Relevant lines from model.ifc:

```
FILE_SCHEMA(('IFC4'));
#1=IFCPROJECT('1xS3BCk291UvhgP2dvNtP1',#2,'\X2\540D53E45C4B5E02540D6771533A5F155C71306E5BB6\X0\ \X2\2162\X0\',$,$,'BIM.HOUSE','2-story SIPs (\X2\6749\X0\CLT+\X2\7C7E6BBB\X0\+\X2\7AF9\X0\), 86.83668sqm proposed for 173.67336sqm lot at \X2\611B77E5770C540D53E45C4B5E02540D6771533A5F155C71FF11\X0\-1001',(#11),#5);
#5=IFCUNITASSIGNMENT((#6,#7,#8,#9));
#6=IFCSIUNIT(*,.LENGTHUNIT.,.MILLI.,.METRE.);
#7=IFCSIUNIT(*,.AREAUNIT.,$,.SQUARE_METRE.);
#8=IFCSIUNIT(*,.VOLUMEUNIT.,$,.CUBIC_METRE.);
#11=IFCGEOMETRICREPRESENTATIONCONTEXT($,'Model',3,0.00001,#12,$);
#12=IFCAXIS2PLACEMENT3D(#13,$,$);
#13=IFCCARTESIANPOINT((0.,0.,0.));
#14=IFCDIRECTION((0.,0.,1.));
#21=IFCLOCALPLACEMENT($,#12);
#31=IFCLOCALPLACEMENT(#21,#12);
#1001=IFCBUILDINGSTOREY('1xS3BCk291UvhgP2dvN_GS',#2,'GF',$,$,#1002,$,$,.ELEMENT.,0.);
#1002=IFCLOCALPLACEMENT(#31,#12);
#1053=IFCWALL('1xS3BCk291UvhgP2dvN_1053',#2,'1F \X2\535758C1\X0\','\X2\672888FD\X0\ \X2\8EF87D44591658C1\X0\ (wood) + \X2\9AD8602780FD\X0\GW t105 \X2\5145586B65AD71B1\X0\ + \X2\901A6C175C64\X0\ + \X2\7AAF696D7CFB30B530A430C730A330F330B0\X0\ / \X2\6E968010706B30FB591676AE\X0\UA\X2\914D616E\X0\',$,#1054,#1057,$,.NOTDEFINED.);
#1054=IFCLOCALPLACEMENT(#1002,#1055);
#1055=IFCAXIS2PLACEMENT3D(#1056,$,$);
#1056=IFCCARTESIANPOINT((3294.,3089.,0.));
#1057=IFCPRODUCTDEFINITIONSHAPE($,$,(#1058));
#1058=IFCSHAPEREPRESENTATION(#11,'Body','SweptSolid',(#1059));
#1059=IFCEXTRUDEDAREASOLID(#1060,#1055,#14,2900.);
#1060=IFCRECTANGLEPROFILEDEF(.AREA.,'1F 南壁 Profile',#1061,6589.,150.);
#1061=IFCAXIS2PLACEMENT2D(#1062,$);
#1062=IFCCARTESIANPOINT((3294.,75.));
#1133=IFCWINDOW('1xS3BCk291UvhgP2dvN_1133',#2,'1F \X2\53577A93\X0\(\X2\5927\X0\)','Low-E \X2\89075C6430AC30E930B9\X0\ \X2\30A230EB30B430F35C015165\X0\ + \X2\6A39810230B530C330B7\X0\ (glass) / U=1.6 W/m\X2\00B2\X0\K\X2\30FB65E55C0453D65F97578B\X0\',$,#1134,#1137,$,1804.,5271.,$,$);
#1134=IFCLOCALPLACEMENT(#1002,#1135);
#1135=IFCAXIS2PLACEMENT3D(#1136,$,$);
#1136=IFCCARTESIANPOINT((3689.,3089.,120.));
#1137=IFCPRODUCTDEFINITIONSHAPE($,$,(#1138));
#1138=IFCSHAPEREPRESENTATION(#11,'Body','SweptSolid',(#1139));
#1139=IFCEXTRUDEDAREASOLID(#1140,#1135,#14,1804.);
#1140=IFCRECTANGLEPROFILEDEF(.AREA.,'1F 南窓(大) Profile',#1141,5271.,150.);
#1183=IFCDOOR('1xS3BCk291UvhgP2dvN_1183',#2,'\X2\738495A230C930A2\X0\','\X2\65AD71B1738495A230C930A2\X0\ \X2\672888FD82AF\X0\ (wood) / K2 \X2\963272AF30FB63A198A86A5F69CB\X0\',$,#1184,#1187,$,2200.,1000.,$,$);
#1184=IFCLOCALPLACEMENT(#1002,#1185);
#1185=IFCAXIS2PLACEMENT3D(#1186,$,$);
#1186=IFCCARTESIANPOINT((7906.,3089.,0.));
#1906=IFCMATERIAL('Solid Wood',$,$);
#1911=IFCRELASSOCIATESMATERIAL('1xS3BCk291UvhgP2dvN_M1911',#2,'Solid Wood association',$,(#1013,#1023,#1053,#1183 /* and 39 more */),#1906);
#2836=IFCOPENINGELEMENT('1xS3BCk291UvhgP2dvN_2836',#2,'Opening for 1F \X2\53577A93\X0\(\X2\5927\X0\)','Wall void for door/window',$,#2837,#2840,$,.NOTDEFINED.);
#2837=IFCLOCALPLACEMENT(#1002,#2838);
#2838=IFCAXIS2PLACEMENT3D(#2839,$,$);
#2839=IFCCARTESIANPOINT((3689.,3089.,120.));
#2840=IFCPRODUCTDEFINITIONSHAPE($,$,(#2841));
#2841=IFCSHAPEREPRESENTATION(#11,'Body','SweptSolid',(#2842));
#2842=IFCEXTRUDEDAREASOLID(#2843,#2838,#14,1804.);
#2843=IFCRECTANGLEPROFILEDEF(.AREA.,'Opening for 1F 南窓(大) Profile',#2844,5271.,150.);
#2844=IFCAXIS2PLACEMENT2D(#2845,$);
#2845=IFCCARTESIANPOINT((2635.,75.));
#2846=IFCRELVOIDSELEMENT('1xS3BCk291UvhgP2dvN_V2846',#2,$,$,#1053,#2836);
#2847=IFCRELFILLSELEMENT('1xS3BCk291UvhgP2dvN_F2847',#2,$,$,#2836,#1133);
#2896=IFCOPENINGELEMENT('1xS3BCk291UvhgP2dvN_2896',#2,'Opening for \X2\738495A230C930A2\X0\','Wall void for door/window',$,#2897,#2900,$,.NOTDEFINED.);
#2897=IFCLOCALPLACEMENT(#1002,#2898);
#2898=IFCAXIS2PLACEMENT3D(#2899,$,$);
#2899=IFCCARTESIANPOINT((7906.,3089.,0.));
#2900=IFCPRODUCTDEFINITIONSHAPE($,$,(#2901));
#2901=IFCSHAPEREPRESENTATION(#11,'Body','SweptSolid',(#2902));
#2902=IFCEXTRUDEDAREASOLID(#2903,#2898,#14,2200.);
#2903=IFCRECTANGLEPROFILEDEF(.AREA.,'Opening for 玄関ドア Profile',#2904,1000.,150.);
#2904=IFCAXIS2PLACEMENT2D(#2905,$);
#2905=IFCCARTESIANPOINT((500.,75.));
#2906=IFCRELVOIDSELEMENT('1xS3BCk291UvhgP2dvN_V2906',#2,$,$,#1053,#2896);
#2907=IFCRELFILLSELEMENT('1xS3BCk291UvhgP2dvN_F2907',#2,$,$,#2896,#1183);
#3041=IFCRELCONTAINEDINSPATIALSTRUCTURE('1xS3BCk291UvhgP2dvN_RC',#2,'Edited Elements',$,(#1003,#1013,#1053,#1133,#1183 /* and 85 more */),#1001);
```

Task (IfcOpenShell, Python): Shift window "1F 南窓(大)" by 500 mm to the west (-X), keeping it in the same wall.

```python
import ifcopenshell
import ifcopenshell.api.geometry
import ifcopenshell.util.placement
import ifcopenshell.util.unit

model = ifcopenshell.open("model.ifc")
unit_scale = ifcopenshell.util.unit.calculate_unit_scale(model)

window = model.by_guid("1xS3BCk291UvhgP2dvN_1133")
opening = window.FillsVoids[0].RelatingOpeningElement
wall = opening.VoidsElements[0].RelatingBuildingElement

wall_matrix = ifcopenshell.util.placement.get_local_placement(wall.ObjectPlacement)
shift = wall_matrix[:3, 0] * -0.5 / unit_scale
before = ifcopenshell.util.placement.get_local_placement(window.ObjectPlacement)[:3, 3].copy()

# The window is not placed relative to its opening, so move both.
for product in (opening, window):
    matrix = ifcopenshell.util.placement.get_local_placement(product.ObjectPlacement)
    matrix[:3, 3] += shift
    ifcopenshell.api.geometry.edit_object_placement(model, product=product, matrix=matrix, is_si=False)

after = ifcopenshell.util.placement.get_local_placement(window.ObjectPlacement)[:3, 3]
print("window moved by", (after - before).round(3) + 0.0)

model.write("model_v2.ifc")
```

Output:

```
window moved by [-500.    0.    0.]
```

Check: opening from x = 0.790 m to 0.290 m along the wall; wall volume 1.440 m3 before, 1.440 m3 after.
